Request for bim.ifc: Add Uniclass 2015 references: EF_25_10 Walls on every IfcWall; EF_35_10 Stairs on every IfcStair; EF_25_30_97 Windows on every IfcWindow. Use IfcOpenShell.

First a look at what the model holds.

```python
import ifcopenshell

model = ifcopenshell.open("bim.ifc")
print(model.schema)
print("classifications:", [c.Name for c in model.by_type("IfcClassification")])
for ifc_class in ("IfcDoor", "IfcRoof", "IfcStair", "IfcWall", "IfcWindow"):
    print(ifc_class, len(model.by_type(ifc_class)))
```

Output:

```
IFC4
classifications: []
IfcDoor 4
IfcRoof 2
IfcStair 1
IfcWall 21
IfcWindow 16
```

```python
import ifcopenshell
import ifcopenshell.api.classification

model = ifcopenshell.open("bim.ifc")

system = ifcopenshell.api.classification.add_classification(model, classification="Uniclass 2015")

codes = {
    "IfcWall": ("EF_25_10", "Walls"),
    "IfcStair": ("EF_35_10", "Stairs"),
    "IfcWindow": ("EF_25_30_97", "Windows"),
}
for ifc_class, (code, name) in codes.items():
    products = model.by_type(ifc_class)
    ifcopenshell.api.classification.add_reference(
        model, products=products, classification=system, identification=code, name=name
    )
    print(code, len(products))

model.write("bim-out.ifc")
```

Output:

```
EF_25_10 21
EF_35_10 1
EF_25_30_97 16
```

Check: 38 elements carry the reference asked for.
